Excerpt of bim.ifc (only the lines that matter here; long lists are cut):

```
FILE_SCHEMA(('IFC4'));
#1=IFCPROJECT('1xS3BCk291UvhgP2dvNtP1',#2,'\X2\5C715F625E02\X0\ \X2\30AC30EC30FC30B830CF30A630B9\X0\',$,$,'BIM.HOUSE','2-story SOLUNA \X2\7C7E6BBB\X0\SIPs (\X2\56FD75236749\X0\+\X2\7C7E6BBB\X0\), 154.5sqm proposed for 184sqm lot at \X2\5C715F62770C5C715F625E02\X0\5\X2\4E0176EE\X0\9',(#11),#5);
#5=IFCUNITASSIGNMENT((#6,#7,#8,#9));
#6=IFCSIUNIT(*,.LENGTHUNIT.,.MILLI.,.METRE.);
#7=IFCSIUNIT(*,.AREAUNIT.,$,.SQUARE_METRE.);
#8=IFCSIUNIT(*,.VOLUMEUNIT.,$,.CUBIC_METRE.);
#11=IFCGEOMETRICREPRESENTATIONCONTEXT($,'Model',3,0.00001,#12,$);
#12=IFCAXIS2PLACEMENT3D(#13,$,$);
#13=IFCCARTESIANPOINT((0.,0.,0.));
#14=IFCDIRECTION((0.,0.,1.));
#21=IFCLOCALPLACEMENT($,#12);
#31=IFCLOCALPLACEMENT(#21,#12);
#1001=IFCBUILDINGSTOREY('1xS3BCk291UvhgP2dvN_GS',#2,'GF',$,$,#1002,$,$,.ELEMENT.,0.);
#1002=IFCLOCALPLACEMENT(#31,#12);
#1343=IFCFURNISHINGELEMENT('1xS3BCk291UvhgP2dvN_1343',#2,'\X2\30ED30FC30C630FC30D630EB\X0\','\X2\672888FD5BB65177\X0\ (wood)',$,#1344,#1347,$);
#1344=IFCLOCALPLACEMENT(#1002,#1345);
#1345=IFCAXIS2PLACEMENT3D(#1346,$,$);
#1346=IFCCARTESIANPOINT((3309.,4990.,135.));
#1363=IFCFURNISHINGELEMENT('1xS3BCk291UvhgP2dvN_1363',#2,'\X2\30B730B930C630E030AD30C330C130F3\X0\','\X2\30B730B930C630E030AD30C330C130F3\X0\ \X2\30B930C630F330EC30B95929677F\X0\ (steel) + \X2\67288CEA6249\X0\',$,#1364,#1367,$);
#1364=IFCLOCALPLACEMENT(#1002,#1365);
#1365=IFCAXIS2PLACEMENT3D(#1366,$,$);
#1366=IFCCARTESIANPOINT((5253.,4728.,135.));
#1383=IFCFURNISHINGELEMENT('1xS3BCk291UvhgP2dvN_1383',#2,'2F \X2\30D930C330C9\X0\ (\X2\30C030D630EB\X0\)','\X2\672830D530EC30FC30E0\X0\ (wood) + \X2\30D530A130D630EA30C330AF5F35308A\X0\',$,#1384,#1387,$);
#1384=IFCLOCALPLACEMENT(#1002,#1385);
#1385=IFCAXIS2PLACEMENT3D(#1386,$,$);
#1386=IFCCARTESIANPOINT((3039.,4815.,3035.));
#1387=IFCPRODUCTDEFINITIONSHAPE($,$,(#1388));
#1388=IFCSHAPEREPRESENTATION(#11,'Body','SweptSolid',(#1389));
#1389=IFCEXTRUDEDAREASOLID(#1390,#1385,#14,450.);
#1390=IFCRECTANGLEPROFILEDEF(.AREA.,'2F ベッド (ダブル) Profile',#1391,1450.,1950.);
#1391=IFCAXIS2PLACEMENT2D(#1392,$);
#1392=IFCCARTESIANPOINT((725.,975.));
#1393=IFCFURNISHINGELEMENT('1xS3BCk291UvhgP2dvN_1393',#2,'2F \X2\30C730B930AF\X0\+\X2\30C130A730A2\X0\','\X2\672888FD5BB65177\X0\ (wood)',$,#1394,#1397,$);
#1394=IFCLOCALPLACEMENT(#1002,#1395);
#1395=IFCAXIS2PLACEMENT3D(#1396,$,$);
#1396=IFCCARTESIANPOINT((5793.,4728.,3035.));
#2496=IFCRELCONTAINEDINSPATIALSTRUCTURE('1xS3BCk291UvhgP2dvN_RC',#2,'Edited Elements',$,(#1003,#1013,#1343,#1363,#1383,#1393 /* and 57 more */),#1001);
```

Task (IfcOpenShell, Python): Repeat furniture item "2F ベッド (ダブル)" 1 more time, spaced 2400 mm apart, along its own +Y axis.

```python
import ifcopenshell
import ifcopenshell.api.geometry
import ifcopenshell.api.root
import ifcopenshell.util.element
import ifcopenshell.util.placement
import ifcopenshell.util.unit

model = ifcopenshell.open("bim.ifc")
unit_scale = ifcopenshell.util.unit.calculate_unit_scale(model)


def reuse_history(source, copy):
    """copy_class also copies each property set's owner history, people and application; keep the originals."""
    for rel in copy.IsDefinedBy:
        if rel.is_a("IfcRelDefinesByProperties") and (history := rel.RelatingPropertyDefinition.OwnerHistory):
            rel.RelatingPropertyDefinition.OwnerHistory = source.OwnerHistory
            ifcopenshell.util.element.remove_deep2(model, history)


source = model.by_id(1383)
base = ifcopenshell.util.placement.get_local_placement(source.ObjectPlacement)
step = base[:3, 1] * 2.4 / unit_scale

for i in range(1, 2):
    copy = ifcopenshell.api.root.copy_class(model, product=source)
    copy.Representation = ifcopenshell.util.element.copy_deep(
        model, source.Representation, exclude=["IfcGeometricRepresentationContext", "IfcRepresentationMap"]
    )
    reuse_history(source, copy)
    matrix = base.copy()
    matrix[:3, 3] += i * step
    print("added at", matrix[:3, 3].round(3) + 0.0)
    ifcopenshell.api.geometry.edit_object_placement(model, product=copy, matrix=matrix, is_si=False)

model.write("bim_edited.ifc")
```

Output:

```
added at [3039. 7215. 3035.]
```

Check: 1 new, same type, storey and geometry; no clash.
